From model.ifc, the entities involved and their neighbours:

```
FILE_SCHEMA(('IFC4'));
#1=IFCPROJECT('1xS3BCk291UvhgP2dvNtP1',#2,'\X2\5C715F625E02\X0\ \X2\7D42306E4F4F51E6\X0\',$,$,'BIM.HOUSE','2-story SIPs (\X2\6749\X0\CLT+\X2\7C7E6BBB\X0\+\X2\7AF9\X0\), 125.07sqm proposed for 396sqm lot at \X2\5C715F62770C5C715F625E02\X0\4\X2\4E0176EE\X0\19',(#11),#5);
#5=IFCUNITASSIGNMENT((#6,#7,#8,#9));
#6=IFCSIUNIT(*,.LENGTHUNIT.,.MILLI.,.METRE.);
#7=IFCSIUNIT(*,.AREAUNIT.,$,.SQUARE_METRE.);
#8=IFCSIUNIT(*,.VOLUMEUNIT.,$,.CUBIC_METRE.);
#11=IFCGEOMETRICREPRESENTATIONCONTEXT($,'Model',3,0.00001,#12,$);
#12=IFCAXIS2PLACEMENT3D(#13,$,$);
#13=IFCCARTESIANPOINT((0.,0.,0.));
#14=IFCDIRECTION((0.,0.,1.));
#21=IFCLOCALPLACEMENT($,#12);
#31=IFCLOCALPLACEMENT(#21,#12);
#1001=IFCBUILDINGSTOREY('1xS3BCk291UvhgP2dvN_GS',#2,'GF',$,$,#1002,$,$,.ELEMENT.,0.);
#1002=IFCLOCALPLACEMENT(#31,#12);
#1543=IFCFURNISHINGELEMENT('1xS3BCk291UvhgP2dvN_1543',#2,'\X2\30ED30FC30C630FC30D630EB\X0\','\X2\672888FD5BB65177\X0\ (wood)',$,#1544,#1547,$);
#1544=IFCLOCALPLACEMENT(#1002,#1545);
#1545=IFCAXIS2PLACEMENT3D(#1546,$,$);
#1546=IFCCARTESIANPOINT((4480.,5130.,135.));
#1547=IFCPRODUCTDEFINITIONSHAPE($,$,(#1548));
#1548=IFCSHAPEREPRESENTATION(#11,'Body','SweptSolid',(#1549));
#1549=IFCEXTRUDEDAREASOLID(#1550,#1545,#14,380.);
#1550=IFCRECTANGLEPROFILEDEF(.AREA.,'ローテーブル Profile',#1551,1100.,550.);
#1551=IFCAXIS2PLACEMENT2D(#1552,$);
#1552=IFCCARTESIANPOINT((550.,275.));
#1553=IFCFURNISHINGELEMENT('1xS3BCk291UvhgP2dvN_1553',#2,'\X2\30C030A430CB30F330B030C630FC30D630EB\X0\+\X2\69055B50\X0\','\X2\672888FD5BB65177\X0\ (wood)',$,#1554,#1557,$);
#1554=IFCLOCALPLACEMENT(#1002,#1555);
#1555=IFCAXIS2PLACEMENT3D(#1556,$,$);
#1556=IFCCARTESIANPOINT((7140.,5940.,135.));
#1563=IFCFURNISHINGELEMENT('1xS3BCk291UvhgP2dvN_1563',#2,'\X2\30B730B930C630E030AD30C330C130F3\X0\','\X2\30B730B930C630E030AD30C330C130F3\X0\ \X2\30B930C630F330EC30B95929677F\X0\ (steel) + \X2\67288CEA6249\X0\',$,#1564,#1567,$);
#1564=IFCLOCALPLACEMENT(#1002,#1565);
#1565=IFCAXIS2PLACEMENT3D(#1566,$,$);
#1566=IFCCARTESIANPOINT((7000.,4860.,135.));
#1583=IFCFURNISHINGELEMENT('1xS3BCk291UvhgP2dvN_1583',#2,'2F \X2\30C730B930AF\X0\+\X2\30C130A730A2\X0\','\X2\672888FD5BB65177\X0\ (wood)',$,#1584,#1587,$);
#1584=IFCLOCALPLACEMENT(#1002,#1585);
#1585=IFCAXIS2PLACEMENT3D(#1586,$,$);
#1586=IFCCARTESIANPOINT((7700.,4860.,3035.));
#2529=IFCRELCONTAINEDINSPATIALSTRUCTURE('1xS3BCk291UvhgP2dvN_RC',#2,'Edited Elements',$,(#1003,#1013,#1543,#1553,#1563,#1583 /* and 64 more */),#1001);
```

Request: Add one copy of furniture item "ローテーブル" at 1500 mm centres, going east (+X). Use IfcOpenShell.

```python
import numpy as np
import ifcopenshell
import ifcopenshell.api.geometry
import ifcopenshell.api.root
import ifcopenshell.util.element
import ifcopenshell.util.placement
import ifcopenshell.util.unit

model = ifcopenshell.open("model.ifc")
unit_scale = ifcopenshell.util.unit.calculate_unit_scale(model)


def reuse_history(source, copy):
    """copy_class also copies each property set's owner history, people and application; keep the originals."""
    for rel in copy.IsDefinedBy:
        if rel.is_a("IfcRelDefinesByProperties") and (history := rel.RelatingPropertyDefinition.OwnerHistory):
            rel.RelatingPropertyDefinition.OwnerHistory = source.OwnerHistory
            ifcopenshell.util.element.remove_deep2(model, history)


source = model.by_guid("1xS3BCk291UvhgP2dvN_1543")
base = ifcopenshell.util.placement.get_local_placement(source.ObjectPlacement)
step = np.array([1.0, 0.0, 0.0]) * 1.5 / unit_scale

for i in range(1, 2):
    copy = ifcopenshell.api.root.copy_class(model, product=source)
    copy.Representation = ifcopenshell.util.element.copy_deep(
        model, source.Representation, exclude=["IfcGeometricRepresentationContext", "IfcRepresentationMap"]
    )
    reuse_history(source, copy)
    matrix = base.copy()
    matrix[:3, 3] += i * step
    print("added at", matrix[:3, 3].round(3) + 0.0)
    ifcopenshell.api.geometry.edit_object_placement(model, product=copy, matrix=matrix, is_si=False)

model.write("model_edited.ifc")
```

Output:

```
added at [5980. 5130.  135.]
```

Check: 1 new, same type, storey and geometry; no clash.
